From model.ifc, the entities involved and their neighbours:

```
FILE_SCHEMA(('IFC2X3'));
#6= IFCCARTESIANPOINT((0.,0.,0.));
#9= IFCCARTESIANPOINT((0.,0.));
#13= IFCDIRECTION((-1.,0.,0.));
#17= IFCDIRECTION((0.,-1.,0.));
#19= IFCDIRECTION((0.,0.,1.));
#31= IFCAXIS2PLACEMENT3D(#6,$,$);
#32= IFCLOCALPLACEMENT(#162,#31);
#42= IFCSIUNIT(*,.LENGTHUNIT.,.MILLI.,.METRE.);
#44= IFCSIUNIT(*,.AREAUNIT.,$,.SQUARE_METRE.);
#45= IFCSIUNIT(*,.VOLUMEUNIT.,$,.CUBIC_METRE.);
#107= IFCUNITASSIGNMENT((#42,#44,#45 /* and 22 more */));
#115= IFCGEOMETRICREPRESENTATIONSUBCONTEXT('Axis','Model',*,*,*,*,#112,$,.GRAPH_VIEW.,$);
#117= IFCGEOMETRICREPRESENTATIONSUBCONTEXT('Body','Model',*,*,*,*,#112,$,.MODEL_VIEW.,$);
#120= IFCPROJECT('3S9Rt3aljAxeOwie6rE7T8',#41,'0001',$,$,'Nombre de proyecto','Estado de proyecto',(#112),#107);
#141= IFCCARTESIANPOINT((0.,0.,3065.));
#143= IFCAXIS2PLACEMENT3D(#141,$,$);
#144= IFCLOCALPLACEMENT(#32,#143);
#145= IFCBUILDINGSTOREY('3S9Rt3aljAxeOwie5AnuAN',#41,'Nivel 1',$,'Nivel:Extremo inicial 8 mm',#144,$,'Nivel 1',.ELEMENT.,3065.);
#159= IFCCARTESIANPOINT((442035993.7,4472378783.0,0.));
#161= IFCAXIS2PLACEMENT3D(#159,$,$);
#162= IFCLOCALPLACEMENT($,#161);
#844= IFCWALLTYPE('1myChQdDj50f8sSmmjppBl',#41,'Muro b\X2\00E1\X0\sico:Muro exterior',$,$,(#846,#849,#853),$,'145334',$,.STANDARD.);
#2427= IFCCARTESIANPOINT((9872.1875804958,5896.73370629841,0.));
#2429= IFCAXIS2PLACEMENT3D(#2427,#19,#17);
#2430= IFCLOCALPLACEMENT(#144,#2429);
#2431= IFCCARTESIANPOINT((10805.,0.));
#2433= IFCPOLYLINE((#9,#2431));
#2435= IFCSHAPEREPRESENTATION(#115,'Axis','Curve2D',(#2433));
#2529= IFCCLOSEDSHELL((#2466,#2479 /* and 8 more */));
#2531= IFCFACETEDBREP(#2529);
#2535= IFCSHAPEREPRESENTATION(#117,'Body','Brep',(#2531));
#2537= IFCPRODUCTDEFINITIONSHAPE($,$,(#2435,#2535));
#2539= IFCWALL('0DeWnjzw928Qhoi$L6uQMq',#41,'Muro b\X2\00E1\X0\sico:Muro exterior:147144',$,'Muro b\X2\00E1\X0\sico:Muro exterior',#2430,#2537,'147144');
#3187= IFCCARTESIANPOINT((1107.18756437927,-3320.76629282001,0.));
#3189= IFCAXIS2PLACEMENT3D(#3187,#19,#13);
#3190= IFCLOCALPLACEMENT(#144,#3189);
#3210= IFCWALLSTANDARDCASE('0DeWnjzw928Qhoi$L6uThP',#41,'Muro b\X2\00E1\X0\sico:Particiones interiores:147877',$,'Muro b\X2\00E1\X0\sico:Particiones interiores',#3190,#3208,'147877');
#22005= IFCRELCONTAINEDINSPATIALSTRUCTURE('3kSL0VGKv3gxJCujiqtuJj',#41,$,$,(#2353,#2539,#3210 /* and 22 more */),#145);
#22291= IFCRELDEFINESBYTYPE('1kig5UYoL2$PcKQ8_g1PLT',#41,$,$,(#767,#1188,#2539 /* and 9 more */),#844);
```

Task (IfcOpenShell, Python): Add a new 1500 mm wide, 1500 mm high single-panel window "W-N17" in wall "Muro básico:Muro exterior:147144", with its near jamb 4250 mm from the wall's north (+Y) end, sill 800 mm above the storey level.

```python
import numpy as np
import ifcopenshell
import ifcopenshell.api.feature
import ifcopenshell.api.geometry
import ifcopenshell.api.root
import ifcopenshell.api.spatial
import ifcopenshell.api.type
import ifcopenshell.geom
import ifcopenshell.util.element
import ifcopenshell.util.placement
import ifcopenshell.util.representation
import ifcopenshell.util.shape
import ifcopenshell.util.unit

model = ifcopenshell.open("model.ifc")
unit_scale = ifcopenshell.util.unit.calculate_unit_scale(model)
settings = ifcopenshell.geom.settings()


def volume(element):
    """Net volume in cubic metres, openings subtracted."""
    shape = ifcopenshell.geom.create_shape(settings, element)
    return ifcopenshell.util.shape.get_volume(shape.geometry)


wall = model.by_guid("0DeWnjzw928Qhoi$L6uQMq")
storey = ifcopenshell.util.element.get_container(wall, ifc_class="IfcBuildingStorey")
context = ifcopenshell.util.representation.get_context(model, "Model", "Body", "MODEL_VIEW")
before = volume(wall)

width, height, from_end, sill = 1.5, 1.5, 4.25, 0.8  # metres

# The wall runs along its own X axis, and the end named is its -X end.
wall_shape = ifcopenshell.geom.create_shape(settings, wall)
x, y, z = ifcopenshell.util.shape.get_vertices(wall_shape.geometry).T
start = x.min() + from_end
face, thickness = float(y.min()), float(y.max() - y.min())
wall_matrix = ifcopenshell.util.placement.get_local_placement(wall.ObjectPlacement)
level = ifcopenshell.util.placement.get_local_placement(storey.ObjectPlacement)[2, 3]


def in_wall(x, y):
    """Placement at x, y metres in the wall's axes, at sill height."""
    matrix = wall_matrix.copy()
    matrix[:, 3] = wall_matrix @ np.array([x / unit_scale, y / unit_scale, 0.0, 1.0])
    matrix[2, 3] = level + sill / unit_scale
    return matrix


# Opening: a box that overshoots both wall faces by 50 mm.
opening = ifcopenshell.api.root.create_entity(model, ifc_class="IfcOpeningElement")
box = ifcopenshell.api.geometry.add_wall_representation(
    model, context=context, length=width, height=height, thickness=thickness + 0.1
)
ifcopenshell.api.geometry.assign_representation(model, product=opening, representation=box)
ifcopenshell.api.geometry.edit_object_placement(model, product=opening, matrix=in_wall(start, face - 0.05), is_si=False)
ifcopenshell.api.feature.add_feature(model, feature=opening, element=wall)

window = ifcopenshell.api.root.create_entity(model, ifc_class="IfcWindow", name="W-N17")
window.OverallWidth, window.OverallHeight = width / unit_scale, height / unit_scale
body = ifcopenshell.api.geometry.add_window_representation(
    model,
    context=context,
    overall_width=window.OverallWidth,
    overall_height=window.OverallHeight,
    partition_type="SINGLE_PANEL",
)
ifcopenshell.api.geometry.assign_representation(model, product=window, representation=body)
ifcopenshell.api.spatial.assign_container(model, products=[window], relating_structure=storey)
fills = ifcopenshell.api.feature.add_filling(model, opening=opening, element=window)
fills.OwnerHistory = window.OwnerHistory  # required in IFC2X3

# IFC2X3 keeps the operation on the window style.
style = ifcopenshell.api.root.create_entity(model, ifc_class="IfcWindowStyle", name="W-N17")
style.OperationType, style.ConstructionType = "SINGLE_PANEL", "NOTDEFINED"
style.ParameterTakesPrecedence = style.Sizeable = False
ifcopenshell.api.type.assign_type(model, related_objects=[window], relating_type=style)

# Centre the window in the wall's thickness.
ifcopenshell.api.geometry.edit_object_placement(model, product=window, matrix=in_wall(start, face), is_si=False)
window_shape = ifcopenshell.geom.create_shape(settings, window)
depth = ifcopenshell.util.shape.get_vertices(window_shape.geometry)[:, 1]
offset = face + thickness / 2 - (depth.min() + depth.max()) / 2
ifcopenshell.api.geometry.edit_object_placement(model, product=window, matrix=in_wall(start, offset), is_si=False)

after = volume(wall)

print(f"wall volume {before:.3f} -> {after:.3f} m3")

model.write("model-out.ifc")
```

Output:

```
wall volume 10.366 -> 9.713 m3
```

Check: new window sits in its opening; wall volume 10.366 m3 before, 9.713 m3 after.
